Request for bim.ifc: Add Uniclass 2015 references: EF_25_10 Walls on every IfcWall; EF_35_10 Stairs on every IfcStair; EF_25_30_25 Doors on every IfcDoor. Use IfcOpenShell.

First a look at what the model holds.

```python
import ifcopenshell

model = ifcopenshell.open("bim.ifc")
print(model.schema)
print("classifications:", [c.Name for c in model.by_type("IfcClassification")])
for ifc_class in ("IfcDoor", "IfcRoof", "IfcStair", "IfcWall", "IfcWindow"):
    print(ifc_class, len(model.by_type(ifc_class)))
```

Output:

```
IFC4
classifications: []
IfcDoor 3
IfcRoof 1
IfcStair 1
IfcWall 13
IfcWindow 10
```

```python
import ifcopenshell
import ifcopenshell.api.classification

model = ifcopenshell.open("bim.ifc")

system = ifcopenshell.api.classification.add_classification(model, classification="Uniclass 2015")

codes = {
    "IfcWall": ("EF_25_10", "Walls"),
    "IfcStair": ("EF_35_10", "Stairs"),
    "IfcDoor": ("EF_25_30_25", "Doors"),
}
for ifc_class, (code, name) in codes.items():
    products = model.by_type(ifc_class)
    ifcopenshell.api.classification.add_reference(
        model, products=products, classification=system, identification=code, name=name
    )
    print(code, len(products))

model.write("bim_edited.ifc")
```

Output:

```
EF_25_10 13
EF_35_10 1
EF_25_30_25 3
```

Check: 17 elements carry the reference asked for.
